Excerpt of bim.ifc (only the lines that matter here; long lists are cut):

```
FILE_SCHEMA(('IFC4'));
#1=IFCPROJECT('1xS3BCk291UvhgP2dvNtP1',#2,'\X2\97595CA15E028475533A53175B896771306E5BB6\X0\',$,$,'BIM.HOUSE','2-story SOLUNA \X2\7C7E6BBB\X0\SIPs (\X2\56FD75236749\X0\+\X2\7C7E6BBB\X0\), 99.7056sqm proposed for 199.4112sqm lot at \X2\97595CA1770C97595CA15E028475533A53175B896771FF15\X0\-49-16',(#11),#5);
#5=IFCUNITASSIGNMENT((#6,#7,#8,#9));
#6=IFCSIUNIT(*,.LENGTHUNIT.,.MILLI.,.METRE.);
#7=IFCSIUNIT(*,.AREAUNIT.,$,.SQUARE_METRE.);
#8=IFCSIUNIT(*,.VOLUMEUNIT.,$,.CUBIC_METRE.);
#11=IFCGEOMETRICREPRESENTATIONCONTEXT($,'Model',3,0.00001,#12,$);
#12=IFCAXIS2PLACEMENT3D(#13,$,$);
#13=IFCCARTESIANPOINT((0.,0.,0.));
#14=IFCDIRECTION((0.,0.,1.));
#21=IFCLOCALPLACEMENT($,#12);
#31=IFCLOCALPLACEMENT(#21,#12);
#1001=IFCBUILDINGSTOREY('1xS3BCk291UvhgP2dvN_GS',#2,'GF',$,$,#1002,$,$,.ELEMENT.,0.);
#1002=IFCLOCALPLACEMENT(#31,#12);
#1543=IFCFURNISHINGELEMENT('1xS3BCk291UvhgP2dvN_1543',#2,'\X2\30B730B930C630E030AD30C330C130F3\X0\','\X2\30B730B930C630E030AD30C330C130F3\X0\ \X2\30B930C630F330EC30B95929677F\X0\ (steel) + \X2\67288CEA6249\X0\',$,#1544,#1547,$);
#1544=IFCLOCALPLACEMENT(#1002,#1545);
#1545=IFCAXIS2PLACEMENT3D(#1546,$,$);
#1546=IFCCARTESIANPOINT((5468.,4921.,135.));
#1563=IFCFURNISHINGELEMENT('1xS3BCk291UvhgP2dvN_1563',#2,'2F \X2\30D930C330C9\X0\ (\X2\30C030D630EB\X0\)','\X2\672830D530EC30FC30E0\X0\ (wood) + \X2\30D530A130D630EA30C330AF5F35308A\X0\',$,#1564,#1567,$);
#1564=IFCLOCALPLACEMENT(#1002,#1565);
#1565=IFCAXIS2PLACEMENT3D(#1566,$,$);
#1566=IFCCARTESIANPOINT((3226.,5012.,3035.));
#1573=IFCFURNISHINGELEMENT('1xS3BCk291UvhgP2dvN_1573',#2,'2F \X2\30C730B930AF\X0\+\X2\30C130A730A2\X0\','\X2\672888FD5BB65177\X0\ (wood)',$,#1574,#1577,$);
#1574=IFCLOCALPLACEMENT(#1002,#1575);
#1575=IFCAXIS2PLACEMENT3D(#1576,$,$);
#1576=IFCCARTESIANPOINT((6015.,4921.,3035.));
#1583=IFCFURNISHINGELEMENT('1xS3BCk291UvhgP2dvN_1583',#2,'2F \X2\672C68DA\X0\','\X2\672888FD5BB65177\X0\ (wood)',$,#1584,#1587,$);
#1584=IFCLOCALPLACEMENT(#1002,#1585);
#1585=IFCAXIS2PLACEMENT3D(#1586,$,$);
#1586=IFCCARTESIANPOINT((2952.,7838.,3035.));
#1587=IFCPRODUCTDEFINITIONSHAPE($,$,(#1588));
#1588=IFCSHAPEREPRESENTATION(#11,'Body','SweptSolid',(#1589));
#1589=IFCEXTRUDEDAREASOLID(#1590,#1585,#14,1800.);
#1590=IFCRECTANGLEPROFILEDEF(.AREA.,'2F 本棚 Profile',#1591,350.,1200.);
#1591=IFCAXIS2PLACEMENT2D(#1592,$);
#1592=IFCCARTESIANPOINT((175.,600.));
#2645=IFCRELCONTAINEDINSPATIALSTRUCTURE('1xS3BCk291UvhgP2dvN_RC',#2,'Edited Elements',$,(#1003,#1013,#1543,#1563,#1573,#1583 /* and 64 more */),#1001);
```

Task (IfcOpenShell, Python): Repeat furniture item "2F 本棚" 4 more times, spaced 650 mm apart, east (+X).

```python
import numpy as np
import ifcopenshell
import ifcopenshell.api.geometry
import ifcopenshell.api.root
import ifcopenshell.util.element
import ifcopenshell.util.placement
import ifcopenshell.util.unit

model = ifcopenshell.open("bim.ifc")
unit_scale = ifcopenshell.util.unit.calculate_unit_scale(model)


def reuse_history(source, copy):
    """copy_class also copies each property set's owner history, people and application; keep the originals."""
    for rel in copy.IsDefinedBy:
        if rel.is_a("IfcRelDefinesByProperties") and (history := rel.RelatingPropertyDefinition.OwnerHistory):
            rel.RelatingPropertyDefinition.OwnerHistory = source.OwnerHistory
            ifcopenshell.util.element.remove_deep2(model, history)


source = model.by_guid("1xS3BCk291UvhgP2dvN_1583")
base = ifcopenshell.util.placement.get_local_placement(source.ObjectPlacement)
step = np.array([1.0, 0.0, 0.0]) * 0.65 / unit_scale

for i in range(1, 5):
    copy = ifcopenshell.api.root.copy_class(model, product=source)
    copy.Representation = ifcopenshell.util.element.copy_deep(
        model, source.Representation, exclude=["IfcGeometricRepresentationContext", "IfcRepresentationMap"]
    )
    reuse_history(source, copy)
    matrix = base.copy()
    matrix[:3, 3] += i * step
    print("added at", matrix[:3, 3].round(3) + 0.0)
    ifcopenshell.api.geometry.edit_object_placement(model, product=copy, matrix=matrix, is_si=False)

model.write("bim_rev.ifc")
```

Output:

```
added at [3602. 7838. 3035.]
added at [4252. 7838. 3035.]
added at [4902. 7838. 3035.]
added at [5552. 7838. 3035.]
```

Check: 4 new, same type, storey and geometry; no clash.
